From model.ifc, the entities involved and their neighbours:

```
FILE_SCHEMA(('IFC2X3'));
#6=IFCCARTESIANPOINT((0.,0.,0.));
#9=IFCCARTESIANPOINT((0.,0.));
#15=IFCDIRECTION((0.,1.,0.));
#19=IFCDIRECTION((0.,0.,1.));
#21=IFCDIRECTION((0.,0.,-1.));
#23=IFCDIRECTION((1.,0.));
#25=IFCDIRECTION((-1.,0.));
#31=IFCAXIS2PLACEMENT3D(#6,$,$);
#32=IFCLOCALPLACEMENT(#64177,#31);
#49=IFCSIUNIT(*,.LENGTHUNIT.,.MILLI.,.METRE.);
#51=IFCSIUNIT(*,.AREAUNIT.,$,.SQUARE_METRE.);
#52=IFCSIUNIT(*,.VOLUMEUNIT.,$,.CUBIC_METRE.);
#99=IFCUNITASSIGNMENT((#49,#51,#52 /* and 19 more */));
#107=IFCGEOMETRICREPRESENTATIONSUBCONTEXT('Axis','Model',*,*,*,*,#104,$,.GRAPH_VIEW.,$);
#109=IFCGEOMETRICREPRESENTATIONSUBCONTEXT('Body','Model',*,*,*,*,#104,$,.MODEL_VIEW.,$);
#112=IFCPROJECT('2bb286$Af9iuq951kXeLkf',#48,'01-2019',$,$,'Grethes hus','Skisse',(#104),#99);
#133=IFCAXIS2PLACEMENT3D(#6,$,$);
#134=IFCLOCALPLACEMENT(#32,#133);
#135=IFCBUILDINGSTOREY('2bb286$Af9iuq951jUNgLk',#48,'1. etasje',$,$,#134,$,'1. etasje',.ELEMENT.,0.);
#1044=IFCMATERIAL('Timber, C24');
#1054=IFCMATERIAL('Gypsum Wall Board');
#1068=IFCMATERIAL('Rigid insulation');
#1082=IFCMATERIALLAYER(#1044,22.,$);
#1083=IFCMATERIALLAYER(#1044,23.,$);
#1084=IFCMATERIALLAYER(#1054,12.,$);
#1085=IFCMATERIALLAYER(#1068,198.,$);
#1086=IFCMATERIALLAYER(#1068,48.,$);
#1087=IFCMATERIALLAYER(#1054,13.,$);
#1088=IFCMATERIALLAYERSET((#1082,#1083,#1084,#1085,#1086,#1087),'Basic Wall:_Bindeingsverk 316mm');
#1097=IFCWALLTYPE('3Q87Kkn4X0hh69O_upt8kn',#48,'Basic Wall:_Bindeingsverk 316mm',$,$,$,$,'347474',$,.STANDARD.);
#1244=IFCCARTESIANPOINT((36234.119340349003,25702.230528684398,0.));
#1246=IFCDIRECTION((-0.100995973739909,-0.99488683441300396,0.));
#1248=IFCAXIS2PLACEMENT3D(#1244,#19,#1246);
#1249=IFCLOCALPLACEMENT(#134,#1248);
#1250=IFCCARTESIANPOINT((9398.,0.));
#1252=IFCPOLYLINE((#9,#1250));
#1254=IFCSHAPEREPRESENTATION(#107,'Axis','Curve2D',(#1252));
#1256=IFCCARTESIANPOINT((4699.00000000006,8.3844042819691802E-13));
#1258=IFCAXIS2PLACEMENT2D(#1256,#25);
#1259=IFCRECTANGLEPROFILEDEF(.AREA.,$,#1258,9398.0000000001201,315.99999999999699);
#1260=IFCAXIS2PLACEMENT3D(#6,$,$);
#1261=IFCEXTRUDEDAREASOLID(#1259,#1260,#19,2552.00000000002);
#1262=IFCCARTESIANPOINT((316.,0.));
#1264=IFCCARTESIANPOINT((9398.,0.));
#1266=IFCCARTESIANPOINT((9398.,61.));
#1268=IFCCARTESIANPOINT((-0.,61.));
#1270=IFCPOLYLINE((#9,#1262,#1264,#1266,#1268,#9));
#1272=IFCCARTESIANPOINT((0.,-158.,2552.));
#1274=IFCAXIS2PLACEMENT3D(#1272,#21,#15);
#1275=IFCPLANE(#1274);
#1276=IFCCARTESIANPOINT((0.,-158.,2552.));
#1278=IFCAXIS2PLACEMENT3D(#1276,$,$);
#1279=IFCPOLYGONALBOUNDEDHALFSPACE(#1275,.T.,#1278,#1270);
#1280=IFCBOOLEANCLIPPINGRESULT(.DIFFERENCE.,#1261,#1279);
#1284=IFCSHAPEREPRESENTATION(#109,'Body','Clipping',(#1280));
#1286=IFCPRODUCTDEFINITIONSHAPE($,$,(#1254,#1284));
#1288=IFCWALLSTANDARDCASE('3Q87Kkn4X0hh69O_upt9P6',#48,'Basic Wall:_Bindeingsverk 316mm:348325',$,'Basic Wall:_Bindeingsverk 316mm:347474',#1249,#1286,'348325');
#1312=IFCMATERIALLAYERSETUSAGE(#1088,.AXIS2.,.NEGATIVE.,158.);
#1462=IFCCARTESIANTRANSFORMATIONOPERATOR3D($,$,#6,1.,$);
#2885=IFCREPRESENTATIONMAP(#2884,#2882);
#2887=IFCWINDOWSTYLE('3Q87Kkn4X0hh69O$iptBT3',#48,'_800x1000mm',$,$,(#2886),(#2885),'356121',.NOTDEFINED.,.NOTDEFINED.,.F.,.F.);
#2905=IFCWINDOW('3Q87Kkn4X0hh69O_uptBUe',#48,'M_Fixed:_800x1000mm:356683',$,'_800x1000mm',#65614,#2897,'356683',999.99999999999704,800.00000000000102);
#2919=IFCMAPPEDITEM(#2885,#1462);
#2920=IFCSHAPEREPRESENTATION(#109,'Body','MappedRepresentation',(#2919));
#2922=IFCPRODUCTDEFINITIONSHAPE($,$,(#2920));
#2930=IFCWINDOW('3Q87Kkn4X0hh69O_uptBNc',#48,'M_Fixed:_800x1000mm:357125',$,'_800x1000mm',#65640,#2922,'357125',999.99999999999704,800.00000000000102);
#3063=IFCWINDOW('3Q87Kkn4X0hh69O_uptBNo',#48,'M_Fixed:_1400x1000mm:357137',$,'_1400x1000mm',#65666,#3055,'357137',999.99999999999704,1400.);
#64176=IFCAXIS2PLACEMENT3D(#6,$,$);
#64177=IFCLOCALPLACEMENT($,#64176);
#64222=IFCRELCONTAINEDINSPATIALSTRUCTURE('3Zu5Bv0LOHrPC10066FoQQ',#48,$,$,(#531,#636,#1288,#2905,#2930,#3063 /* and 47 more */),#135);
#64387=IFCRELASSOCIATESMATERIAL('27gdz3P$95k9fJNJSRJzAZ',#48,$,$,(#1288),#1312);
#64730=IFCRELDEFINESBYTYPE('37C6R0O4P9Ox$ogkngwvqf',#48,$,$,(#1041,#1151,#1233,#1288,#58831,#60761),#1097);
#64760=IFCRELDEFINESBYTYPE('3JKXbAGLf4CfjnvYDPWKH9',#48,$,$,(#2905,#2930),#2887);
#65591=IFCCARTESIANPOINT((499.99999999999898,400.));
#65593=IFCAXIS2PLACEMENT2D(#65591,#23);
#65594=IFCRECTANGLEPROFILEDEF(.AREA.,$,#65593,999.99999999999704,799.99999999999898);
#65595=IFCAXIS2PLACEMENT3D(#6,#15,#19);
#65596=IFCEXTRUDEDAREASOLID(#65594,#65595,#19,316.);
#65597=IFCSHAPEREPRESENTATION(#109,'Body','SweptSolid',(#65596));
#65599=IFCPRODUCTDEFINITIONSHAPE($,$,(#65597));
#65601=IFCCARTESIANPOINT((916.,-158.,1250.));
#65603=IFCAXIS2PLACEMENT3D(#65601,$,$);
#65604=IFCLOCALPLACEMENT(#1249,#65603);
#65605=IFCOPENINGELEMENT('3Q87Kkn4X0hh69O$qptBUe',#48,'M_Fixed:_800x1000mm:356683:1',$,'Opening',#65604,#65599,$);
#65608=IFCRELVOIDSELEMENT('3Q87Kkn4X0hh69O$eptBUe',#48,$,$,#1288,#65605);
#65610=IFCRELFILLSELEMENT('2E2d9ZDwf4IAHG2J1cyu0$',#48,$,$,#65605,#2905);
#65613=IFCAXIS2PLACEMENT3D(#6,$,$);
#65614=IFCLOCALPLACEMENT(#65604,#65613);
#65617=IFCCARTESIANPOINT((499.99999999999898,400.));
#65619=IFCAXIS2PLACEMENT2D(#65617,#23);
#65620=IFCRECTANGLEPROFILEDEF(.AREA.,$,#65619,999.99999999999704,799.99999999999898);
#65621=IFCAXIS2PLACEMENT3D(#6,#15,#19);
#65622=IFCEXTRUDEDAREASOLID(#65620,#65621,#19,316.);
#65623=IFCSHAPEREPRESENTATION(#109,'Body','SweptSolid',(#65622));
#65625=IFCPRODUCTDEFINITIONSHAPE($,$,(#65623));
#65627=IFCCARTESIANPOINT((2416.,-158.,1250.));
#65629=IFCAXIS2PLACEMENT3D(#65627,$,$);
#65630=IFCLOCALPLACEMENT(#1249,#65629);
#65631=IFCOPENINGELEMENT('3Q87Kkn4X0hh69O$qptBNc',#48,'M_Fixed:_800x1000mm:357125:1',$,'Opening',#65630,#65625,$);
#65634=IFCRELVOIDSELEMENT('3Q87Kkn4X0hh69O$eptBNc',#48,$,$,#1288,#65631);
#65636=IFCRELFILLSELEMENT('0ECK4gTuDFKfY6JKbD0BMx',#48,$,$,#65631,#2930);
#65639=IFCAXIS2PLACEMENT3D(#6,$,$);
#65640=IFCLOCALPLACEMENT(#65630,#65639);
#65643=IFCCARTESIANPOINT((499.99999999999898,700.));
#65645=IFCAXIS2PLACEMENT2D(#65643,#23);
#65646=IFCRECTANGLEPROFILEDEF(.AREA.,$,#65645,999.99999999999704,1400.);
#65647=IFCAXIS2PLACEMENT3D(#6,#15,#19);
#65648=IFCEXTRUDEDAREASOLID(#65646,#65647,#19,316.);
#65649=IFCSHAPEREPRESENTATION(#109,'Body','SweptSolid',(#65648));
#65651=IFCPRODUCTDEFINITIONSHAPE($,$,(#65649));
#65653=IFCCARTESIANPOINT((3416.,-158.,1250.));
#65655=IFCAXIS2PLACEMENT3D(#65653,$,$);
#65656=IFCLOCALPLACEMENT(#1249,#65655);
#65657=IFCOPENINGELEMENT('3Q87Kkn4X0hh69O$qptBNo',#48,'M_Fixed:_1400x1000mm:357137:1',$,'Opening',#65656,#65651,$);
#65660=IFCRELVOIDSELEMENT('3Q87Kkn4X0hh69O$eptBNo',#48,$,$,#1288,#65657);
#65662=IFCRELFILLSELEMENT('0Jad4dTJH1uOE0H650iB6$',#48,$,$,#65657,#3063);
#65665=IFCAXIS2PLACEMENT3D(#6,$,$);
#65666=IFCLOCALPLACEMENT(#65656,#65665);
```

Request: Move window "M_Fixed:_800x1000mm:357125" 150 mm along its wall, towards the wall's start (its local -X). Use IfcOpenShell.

```python
import ifcopenshell
import ifcopenshell.api.geometry
import ifcopenshell.util.placement

model = ifcopenshell.open("model.ifc")

window = model.by_guid("3Q87Kkn4X0hh69O_uptBNc")
opening = window.FillsVoids[0].RelatingOpeningElement
wall = opening.VoidsElements[0].RelatingBuildingElement

wall_matrix = ifcopenshell.util.placement.get_local_placement(wall.ObjectPlacement)
shift = wall_matrix[:3, 0] * -150.0
before = ifcopenshell.util.placement.get_local_placement(window.ObjectPlacement)[:3, 3].copy()

# The window is placed relative to its opening, so it follows when the opening moves.
matrix = ifcopenshell.util.placement.get_local_placement(opening.ObjectPlacement)
matrix[:3, 3] += shift
ifcopenshell.api.geometry.edit_object_placement(
    model, product=opening, matrix=matrix, is_si=False, should_transform_children=True
)

after = ifcopenshell.util.placement.get_local_placement(window.ObjectPlacement)[:3, 3]
print("window moved by", (after - before).round(3) + 0.0)

model.write("model-out.ifc")
```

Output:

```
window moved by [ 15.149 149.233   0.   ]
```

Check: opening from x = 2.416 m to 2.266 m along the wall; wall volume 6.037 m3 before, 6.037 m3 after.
